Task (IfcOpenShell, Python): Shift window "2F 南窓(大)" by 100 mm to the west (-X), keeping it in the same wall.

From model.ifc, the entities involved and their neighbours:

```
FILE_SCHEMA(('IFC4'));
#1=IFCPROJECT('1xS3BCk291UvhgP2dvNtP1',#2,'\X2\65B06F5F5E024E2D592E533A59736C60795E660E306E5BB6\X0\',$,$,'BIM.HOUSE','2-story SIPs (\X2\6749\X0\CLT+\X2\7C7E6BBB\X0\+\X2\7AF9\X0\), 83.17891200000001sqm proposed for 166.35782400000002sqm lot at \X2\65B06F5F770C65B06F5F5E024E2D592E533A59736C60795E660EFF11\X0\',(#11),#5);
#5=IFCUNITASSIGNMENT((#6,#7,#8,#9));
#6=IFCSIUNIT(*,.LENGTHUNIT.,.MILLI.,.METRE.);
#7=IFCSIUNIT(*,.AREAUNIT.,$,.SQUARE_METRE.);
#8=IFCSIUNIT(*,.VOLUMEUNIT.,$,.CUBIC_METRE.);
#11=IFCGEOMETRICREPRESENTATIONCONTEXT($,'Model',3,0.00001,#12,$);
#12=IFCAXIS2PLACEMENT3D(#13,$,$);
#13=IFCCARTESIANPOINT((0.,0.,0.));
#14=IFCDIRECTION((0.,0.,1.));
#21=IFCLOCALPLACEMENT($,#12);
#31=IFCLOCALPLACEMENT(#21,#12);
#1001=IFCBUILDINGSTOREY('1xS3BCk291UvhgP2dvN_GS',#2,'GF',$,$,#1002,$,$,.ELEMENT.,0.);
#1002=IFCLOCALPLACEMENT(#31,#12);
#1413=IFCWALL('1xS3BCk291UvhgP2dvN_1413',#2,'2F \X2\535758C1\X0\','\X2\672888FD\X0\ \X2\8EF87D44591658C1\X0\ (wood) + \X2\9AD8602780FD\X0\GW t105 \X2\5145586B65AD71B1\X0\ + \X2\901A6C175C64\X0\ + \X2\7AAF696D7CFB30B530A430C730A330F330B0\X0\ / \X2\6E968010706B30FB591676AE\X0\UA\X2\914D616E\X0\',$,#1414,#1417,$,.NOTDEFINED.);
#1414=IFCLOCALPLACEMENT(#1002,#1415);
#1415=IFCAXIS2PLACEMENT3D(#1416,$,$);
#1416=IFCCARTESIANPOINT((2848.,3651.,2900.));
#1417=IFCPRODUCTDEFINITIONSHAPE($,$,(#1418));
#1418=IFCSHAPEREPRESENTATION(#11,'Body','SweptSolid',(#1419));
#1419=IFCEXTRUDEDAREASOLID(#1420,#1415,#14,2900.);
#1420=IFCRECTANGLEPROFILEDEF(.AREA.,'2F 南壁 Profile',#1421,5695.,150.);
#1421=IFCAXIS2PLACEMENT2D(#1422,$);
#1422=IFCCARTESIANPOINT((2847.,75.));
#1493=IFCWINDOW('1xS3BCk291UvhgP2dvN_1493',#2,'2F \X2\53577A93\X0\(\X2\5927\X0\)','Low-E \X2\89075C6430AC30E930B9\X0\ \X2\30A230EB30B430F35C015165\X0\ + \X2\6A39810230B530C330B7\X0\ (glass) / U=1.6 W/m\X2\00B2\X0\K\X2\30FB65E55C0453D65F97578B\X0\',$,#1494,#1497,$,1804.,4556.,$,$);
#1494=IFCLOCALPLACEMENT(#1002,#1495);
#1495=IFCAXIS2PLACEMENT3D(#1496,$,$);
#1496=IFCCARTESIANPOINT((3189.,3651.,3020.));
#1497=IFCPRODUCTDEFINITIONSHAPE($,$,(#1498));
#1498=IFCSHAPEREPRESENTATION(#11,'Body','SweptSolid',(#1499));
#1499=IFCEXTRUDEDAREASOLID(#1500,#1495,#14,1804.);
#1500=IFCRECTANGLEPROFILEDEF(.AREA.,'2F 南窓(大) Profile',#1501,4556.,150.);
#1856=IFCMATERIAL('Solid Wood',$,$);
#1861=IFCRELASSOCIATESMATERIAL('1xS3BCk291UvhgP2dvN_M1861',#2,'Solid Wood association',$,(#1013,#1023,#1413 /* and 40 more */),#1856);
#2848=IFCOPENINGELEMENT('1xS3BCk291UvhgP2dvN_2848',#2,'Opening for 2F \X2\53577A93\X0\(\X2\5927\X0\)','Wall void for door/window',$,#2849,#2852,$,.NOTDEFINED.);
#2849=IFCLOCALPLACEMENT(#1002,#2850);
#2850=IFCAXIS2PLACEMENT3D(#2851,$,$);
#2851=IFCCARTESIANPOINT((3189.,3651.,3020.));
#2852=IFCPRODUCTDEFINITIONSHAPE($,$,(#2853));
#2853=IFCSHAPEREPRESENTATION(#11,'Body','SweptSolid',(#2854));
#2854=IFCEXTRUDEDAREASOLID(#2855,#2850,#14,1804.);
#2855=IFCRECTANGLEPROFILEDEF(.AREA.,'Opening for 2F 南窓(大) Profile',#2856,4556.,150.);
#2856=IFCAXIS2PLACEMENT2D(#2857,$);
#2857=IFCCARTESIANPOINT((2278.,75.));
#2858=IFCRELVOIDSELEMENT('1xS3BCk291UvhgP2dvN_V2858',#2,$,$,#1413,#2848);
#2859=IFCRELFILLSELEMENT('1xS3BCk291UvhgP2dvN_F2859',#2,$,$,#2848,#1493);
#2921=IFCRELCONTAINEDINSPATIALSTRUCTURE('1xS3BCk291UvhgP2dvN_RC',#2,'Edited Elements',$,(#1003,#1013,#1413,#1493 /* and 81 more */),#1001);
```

```python
import ifcopenshell
import ifcopenshell.api.geometry
import ifcopenshell.util.placement
import ifcopenshell.util.unit

model = ifcopenshell.open("model.ifc")
unit_scale = ifcopenshell.util.unit.calculate_unit_scale(model)

window = model.by_id(1493)
opening = window.FillsVoids[0].RelatingOpeningElement
wall = opening.VoidsElements[0].RelatingBuildingElement

wall_matrix = ifcopenshell.util.placement.get_local_placement(wall.ObjectPlacement)
shift = wall_matrix[:3, 0] * -0.1 / unit_scale
before = ifcopenshell.util.placement.get_local_placement(window.ObjectPlacement)[:3, 3].copy()

# The window is not placed relative to its opening, so move both.
for product in (opening, window):
    matrix = ifcopenshell.util.placement.get_local_placement(product.ObjectPlacement)
    matrix[:3, 3] += shift
    ifcopenshell.api.geometry.edit_object_placement(model, product=product, matrix=matrix, is_si=False)

after = ifcopenshell.util.placement.get_local_placement(window.ObjectPlacement)[:3, 3]
print("window moved by", (after - before).round(3) + 0.0)

model.write("model-out.ifc")
```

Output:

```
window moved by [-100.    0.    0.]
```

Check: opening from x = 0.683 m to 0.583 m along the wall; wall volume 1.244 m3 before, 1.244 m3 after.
